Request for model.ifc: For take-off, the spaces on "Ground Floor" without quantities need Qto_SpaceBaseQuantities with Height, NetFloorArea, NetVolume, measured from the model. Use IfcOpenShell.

First a look at what the model holds.

```python
import ifcopenshell
import ifcopenshell.util.element
import ifcopenshell.util.unit

model = ifcopenshell.open("model.ifc")
print(model.schema)
for unit_type in ("LENGTHUNIT", "AREAUNIT", "VOLUMEUNIT"):
    print(unit_type, ifcopenshell.util.unit.calculate_unit_scale(model, unit_type))
storey = next(s for s in model.by_type("IfcBuildingStorey") if s.Name == "Ground Floor")
spaces = [e for e in ifcopenshell.util.element.get_decomposition(storey) if e.is_a("IfcSpace")]
for e in sorted(spaces, key=lambda e: e.id()):
    print(e.id(), e.is_a(), e.Name, list(ifcopenshell.util.element.get_psets(e, qtos_only=True)), sep=" | ")
```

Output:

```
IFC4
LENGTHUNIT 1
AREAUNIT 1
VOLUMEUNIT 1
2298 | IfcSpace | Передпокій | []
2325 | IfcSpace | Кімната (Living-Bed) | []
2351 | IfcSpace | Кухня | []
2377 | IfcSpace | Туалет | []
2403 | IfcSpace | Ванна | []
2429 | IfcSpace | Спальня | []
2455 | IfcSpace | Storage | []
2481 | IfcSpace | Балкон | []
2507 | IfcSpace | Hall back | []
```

```python
import ifcopenshell
import ifcopenshell.api.pset
import ifcopenshell.geom
import ifcopenshell.util.element
import ifcopenshell.util.shape
import ifcopenshell.util.unit

model = ifcopenshell.open("model.ifc")
unit_scale = ifcopenshell.util.unit.calculate_unit_scale(model)
area_scale = ifcopenshell.util.unit.calculate_unit_scale(model, "AREAUNIT")
volume_scale = ifcopenshell.util.unit.calculate_unit_scale(model, "VOLUMEUNIT")
settings = ifcopenshell.geom.settings()

storey = next(s for s in model.by_type("IfcBuildingStorey") if s.Name == "Ground Floor")
spaces = [e for e in ifcopenshell.util.element.get_decomposition(storey) if e.is_a("IfcSpace")]

for e in sorted(spaces, key=lambda e: e.id()):
    if ifcopenshell.util.element.get_psets(e, qtos_only=True, should_inherit=False):
        continue
    # Geometry comes back in metres, in the element's own axes.
    shape = ifcopenshell.geom.create_shape(settings, e)
    values = {
        "Height": ifcopenshell.util.shape.get_z(shape.geometry) / unit_scale,
        "NetFloorArea": ifcopenshell.util.shape.get_footprint_area(shape.geometry) / area_scale,
        "NetVolume": ifcopenshell.util.shape.get_volume(shape.geometry) / volume_scale,
    }
    qto = ifcopenshell.api.pset.add_qto(model, product=e, name="Qto_SpaceBaseQuantities")
    ifcopenshell.api.pset.edit_qto(model, qto=qto, properties=values)
    print(e.id(), {k: round(v, 3) for k, v in values.items()})

model.write("model_v2.ifc")
```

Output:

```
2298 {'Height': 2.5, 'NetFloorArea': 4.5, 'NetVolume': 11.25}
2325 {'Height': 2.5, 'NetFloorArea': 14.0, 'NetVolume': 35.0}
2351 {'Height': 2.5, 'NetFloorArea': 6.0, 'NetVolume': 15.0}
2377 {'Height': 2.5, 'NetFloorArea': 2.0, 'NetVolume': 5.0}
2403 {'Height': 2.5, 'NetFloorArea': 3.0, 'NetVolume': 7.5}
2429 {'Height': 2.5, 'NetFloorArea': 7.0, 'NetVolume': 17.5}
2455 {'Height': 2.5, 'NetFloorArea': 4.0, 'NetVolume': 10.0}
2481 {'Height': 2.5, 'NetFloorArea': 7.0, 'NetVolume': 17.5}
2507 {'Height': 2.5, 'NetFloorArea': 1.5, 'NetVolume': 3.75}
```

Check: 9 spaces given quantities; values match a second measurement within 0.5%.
